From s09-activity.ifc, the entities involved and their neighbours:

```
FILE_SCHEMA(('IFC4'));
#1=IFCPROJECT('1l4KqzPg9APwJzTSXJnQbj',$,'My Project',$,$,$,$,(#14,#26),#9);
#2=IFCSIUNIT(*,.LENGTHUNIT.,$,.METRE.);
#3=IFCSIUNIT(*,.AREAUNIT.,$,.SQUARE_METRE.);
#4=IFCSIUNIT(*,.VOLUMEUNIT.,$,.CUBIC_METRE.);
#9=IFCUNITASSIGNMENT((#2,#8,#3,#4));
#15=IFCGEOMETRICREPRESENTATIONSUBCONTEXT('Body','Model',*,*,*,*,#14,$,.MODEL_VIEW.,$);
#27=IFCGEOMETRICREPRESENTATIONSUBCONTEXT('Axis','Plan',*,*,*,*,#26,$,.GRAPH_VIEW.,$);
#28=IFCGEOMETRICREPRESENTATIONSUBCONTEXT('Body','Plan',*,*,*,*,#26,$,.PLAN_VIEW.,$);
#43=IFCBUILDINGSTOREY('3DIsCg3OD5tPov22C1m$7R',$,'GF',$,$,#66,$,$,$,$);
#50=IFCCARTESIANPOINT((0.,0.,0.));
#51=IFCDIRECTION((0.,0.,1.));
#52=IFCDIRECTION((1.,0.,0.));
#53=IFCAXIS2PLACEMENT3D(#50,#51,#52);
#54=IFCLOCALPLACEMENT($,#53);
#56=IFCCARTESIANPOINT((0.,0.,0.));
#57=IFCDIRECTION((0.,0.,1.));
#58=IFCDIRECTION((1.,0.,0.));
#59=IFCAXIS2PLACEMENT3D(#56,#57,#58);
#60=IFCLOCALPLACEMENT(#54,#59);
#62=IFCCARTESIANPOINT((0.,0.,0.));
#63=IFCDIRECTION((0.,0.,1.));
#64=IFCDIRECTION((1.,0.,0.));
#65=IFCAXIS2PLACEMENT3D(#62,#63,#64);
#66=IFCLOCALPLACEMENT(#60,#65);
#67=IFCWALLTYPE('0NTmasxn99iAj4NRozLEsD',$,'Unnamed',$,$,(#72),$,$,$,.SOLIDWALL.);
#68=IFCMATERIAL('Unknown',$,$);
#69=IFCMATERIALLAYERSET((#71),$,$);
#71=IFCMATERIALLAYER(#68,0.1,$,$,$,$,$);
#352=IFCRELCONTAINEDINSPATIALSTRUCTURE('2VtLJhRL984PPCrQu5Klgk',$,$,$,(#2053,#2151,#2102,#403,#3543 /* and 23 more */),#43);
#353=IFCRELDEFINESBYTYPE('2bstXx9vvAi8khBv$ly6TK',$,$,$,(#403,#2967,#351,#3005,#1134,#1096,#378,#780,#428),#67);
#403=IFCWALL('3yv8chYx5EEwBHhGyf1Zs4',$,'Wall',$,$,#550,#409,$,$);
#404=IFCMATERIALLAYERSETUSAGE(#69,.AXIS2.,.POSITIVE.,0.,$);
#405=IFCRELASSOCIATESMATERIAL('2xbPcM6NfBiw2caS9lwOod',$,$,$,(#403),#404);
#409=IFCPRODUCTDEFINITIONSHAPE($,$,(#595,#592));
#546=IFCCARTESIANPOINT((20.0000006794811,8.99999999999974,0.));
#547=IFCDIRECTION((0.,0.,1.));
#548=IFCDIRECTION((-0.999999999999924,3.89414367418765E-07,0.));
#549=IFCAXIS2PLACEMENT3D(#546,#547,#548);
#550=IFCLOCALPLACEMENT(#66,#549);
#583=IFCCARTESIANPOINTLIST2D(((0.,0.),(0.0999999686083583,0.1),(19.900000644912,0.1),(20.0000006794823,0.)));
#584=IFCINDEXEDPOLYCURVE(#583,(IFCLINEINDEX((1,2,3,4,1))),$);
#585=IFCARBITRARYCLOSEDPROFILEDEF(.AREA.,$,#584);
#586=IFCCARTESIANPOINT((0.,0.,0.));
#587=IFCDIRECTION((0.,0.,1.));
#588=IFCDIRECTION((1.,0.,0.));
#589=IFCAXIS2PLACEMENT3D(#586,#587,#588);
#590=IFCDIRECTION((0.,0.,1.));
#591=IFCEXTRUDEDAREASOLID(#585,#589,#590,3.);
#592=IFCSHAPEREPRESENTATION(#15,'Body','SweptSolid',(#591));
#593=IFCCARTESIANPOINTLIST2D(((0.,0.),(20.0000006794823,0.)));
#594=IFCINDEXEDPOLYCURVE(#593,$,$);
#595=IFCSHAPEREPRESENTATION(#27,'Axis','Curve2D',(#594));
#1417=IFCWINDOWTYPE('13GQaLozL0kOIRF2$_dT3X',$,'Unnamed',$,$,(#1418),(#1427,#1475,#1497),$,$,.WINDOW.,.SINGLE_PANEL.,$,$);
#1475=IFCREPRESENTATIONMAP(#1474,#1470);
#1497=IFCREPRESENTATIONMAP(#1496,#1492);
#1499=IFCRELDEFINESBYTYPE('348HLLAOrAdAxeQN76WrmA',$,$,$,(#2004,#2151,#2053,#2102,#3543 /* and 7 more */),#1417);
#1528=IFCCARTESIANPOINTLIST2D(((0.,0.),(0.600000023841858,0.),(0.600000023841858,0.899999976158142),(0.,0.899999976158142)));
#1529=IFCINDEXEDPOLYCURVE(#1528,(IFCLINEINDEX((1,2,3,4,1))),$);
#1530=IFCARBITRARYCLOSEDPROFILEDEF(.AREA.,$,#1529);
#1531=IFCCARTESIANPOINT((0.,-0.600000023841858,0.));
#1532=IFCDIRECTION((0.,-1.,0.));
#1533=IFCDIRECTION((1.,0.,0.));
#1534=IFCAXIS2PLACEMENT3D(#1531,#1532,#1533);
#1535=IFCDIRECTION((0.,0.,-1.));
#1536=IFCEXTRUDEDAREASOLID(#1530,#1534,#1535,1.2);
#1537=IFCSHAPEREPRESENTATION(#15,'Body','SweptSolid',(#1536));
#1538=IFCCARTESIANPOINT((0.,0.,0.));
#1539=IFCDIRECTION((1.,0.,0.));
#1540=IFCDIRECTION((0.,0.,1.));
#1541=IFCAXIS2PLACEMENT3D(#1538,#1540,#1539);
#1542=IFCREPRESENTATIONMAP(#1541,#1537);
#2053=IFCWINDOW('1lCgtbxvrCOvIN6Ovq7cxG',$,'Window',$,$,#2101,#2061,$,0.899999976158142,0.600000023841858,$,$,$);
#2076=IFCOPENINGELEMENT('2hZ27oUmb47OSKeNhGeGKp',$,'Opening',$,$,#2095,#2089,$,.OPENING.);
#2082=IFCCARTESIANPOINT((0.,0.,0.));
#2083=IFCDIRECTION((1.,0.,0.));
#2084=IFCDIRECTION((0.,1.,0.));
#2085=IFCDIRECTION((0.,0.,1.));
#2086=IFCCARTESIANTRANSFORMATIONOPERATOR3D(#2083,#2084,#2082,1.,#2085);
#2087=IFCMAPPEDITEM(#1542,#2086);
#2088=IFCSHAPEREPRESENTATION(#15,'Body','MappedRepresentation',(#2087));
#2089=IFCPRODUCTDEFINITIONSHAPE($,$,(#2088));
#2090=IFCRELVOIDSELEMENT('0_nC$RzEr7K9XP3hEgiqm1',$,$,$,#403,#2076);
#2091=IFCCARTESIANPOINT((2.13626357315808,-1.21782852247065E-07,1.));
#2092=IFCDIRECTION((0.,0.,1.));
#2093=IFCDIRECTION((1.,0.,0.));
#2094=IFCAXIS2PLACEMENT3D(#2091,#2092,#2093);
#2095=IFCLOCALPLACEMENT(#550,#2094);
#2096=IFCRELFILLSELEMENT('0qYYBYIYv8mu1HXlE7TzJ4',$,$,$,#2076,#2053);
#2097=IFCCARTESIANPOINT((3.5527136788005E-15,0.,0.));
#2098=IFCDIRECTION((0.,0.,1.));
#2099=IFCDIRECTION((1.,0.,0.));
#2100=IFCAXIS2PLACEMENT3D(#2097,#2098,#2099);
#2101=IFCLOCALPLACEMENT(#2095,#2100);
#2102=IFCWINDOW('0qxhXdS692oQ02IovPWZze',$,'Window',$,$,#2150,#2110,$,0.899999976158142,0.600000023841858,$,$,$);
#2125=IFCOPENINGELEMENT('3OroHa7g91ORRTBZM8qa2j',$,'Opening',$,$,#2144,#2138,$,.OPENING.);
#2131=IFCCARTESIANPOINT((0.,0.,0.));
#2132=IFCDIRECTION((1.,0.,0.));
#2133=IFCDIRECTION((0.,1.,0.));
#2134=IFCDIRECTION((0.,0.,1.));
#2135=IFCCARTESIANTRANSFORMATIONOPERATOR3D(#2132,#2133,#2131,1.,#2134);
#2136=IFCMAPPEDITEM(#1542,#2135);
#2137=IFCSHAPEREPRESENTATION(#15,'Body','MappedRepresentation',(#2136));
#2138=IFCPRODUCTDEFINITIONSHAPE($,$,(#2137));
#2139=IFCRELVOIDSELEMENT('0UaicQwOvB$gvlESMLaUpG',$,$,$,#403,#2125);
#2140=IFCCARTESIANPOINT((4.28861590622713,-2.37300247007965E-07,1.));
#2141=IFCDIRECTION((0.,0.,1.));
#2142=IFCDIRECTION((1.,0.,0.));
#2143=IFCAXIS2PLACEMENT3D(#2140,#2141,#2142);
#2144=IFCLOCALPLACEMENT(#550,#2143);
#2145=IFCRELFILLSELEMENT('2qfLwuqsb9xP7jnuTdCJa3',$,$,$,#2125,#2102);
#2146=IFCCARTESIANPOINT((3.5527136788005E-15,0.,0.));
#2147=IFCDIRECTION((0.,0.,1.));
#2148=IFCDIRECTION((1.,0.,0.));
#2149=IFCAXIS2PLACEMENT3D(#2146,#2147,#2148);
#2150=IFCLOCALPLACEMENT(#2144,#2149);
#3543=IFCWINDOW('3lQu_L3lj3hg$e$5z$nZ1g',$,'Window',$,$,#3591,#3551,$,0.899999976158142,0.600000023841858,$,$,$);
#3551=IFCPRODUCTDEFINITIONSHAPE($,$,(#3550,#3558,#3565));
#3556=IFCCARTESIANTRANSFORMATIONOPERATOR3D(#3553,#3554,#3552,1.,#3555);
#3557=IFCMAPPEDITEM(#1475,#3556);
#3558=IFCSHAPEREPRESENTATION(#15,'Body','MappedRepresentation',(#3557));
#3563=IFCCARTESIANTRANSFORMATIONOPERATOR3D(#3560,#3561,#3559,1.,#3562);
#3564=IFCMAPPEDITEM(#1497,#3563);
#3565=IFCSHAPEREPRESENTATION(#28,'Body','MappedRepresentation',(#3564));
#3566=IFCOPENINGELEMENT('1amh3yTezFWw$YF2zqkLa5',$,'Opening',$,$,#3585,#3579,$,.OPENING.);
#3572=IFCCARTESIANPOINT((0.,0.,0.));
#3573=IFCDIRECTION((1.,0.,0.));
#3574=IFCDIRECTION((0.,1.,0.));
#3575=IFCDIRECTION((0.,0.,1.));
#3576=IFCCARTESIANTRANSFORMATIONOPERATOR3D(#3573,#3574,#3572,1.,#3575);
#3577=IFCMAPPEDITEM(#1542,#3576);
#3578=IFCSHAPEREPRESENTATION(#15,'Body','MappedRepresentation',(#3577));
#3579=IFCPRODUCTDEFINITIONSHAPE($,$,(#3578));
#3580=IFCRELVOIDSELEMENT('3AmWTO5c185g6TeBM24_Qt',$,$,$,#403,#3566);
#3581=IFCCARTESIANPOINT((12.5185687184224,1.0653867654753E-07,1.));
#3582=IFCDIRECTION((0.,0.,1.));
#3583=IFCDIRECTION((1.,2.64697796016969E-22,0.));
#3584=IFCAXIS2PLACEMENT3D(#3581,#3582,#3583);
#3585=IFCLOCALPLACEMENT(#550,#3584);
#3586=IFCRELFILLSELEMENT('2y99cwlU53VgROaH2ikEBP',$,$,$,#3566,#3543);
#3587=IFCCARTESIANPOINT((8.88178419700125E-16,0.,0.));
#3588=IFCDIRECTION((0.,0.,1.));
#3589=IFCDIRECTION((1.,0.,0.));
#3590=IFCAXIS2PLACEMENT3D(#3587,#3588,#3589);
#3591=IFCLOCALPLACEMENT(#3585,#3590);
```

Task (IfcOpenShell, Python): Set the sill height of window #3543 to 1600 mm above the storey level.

```python
import numpy as np
import ifcopenshell
import ifcopenshell.api.geometry
import ifcopenshell.geom
import ifcopenshell.util.element
import ifcopenshell.util.placement
import ifcopenshell.util.shape
import ifcopenshell.util.unit

model = ifcopenshell.open("s09-activity.ifc")
unit_scale = ifcopenshell.util.unit.calculate_unit_scale(model)

window = model.by_guid("3lQu_L3lj3hg$e$5z$nZ1g")
opening = window.FillsVoids[0].RelatingOpeningElement
storey = ifcopenshell.util.element.get_container(window, ifc_class="IfcBuildingStorey")
level = ifcopenshell.util.placement.get_local_placement(storey.ObjectPlacement)[2, 3]

# The opening's origin need not be at the sill, so measure its lowest point.
shape = ifcopenshell.geom.create_shape(ifcopenshell.geom.settings(), opening)
bottom = ifcopenshell.util.shape.get_shape_bottom_elevation(shape, shape.geometry) / unit_scale
dz = level + 1.6 / unit_scale - bottom

shift = np.array([0.0, 0.0, dz])
# The window is placed relative to its opening, so it follows when the opening moves.
matrix = ifcopenshell.util.placement.get_local_placement(opening.ObjectPlacement)
matrix[:3, 3] += shift
ifcopenshell.api.geometry.edit_object_placement(
    model, product=opening, matrix=matrix, is_si=False, should_transform_children=True
)

print(f"moved by {dz * unit_scale:+.3f} m")

model.write("s09-activity_v2.ifc")
```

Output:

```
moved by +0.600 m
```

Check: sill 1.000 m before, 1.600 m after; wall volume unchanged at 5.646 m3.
